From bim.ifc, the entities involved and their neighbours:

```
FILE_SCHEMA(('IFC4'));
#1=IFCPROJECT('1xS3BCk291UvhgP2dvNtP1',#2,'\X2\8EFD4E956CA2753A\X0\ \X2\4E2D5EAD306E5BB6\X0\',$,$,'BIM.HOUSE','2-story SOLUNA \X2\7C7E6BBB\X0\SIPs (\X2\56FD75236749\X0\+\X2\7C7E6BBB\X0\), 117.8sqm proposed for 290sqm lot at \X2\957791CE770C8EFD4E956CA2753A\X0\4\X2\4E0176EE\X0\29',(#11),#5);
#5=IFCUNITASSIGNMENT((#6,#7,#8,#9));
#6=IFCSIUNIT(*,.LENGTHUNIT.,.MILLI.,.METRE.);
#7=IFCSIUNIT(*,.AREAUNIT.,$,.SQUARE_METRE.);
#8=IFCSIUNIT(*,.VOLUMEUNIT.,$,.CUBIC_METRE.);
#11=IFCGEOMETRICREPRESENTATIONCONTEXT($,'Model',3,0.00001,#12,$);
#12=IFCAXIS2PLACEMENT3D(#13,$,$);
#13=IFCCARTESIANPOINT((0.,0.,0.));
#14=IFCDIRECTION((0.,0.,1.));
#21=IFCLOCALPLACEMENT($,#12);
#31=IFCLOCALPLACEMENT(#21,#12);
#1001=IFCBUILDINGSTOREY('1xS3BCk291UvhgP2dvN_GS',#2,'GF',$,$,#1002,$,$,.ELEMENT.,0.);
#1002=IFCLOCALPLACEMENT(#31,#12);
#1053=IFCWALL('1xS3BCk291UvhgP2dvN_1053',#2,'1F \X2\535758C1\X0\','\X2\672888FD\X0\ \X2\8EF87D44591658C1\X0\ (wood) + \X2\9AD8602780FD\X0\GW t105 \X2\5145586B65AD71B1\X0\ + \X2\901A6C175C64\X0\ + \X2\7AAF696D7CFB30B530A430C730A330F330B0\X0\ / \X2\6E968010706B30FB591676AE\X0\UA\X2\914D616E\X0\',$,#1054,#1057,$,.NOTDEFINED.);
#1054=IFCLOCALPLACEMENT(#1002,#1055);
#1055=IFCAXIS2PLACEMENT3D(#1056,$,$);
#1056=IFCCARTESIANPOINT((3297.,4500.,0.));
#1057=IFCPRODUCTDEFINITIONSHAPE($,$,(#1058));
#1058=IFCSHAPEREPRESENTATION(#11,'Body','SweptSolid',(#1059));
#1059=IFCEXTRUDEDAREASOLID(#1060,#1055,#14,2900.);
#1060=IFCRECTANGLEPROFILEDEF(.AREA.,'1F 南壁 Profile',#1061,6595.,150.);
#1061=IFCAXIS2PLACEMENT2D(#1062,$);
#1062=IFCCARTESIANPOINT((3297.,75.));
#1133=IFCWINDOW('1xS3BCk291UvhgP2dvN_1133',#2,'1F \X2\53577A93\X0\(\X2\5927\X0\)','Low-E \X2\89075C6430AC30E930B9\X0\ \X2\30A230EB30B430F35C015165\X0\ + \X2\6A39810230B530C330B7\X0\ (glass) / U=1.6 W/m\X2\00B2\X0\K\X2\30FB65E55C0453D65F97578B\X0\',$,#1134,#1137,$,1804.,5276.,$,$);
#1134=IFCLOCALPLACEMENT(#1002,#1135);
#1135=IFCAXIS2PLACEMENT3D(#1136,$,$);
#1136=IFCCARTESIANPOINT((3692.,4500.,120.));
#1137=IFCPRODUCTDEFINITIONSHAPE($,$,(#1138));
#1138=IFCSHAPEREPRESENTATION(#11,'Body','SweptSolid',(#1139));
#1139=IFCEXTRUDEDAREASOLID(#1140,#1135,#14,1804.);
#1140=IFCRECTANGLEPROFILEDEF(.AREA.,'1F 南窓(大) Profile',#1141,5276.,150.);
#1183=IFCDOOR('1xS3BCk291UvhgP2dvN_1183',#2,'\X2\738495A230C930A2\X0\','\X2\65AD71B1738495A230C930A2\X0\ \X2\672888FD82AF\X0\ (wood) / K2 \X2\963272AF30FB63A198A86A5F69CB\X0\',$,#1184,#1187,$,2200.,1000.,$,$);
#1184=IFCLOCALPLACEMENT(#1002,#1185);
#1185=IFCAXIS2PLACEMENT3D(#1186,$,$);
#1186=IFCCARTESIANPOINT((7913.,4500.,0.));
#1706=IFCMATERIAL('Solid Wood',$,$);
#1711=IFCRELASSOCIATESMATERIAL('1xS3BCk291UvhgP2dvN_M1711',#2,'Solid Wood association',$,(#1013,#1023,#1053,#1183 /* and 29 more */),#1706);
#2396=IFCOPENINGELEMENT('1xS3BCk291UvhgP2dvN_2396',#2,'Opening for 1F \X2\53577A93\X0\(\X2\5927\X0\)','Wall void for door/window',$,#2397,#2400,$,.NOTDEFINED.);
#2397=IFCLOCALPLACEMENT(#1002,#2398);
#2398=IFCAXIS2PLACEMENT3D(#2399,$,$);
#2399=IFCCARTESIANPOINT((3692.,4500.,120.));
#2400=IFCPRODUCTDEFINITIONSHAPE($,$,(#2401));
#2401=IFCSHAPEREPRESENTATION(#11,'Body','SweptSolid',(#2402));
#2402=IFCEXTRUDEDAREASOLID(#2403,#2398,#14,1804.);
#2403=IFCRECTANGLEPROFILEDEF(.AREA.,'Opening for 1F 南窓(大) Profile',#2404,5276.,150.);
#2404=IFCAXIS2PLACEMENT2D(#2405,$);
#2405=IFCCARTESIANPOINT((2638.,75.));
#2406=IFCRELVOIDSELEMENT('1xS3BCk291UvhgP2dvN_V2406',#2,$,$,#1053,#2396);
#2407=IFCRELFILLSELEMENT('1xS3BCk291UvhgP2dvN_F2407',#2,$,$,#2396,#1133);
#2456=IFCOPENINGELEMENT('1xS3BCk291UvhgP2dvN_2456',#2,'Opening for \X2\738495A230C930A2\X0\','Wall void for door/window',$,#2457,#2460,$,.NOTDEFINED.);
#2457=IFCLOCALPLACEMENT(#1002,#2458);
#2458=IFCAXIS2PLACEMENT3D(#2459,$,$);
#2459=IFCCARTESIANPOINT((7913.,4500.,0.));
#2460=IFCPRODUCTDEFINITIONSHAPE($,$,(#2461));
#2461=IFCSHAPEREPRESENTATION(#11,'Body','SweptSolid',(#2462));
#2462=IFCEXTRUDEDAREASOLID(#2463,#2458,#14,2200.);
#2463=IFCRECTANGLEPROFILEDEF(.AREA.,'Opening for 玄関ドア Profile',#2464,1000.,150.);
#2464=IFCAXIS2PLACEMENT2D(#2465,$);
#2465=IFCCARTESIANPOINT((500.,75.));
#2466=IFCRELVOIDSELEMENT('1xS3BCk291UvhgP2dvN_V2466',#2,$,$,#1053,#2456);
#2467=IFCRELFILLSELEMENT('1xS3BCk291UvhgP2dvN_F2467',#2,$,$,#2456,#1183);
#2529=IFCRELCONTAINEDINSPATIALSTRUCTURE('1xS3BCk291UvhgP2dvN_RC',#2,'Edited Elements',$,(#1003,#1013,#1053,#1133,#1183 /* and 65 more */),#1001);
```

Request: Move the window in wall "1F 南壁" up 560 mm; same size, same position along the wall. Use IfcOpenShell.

```python
import numpy as np
import ifcopenshell
import ifcopenshell.api.geometry
import ifcopenshell.util.placement
import ifcopenshell.util.unit

model = ifcopenshell.open("bim.ifc")
unit_scale = ifcopenshell.util.unit.calculate_unit_scale(model)

window = model.by_guid("1xS3BCk291UvhgP2dvN_1133")
opening = window.FillsVoids[0].RelatingOpeningElement
dz = 0.56 / unit_scale

shift = np.array([0.0, 0.0, dz])
# The window is not placed relative to its opening, so move both.
for product in (opening, window):
    matrix = ifcopenshell.util.placement.get_local_placement(product.ObjectPlacement)
    matrix[:3, 3] += shift
    ifcopenshell.api.geometry.edit_object_placement(model, product=product, matrix=matrix, is_si=False)

print(f"moved by {dz * unit_scale:+.3f} m")

model.write("bim_v2.ifc")
```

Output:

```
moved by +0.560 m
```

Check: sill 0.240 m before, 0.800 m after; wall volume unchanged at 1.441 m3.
